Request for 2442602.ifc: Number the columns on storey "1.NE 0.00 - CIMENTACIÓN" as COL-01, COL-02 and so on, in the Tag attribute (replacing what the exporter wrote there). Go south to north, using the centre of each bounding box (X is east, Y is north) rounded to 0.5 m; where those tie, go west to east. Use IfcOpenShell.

First a look at what the model holds.

```python
import ifcopenshell
import ifcopenshell.util.element
import ifcopenshell.util.placement

model = ifcopenshell.open("2442602.ifc")
print(model.schema)
storey = next(s for s in model.by_type("IfcBuildingStorey") if s.Name == "1.NE 0.00 - CIMENTACIÓN")
columns = [e for e in ifcopenshell.util.element.get_decomposition(storey) if e.is_a("IfcColumn")]
for e in sorted(columns, key=lambda e: e.id()):
    origin = ifcopenshell.util.placement.get_local_placement(e.ObjectPlacement)[:3, 3]
    print(e.id(), e.Tag, e.Name, origin.round(2) + 0.0, sep=" | ")
```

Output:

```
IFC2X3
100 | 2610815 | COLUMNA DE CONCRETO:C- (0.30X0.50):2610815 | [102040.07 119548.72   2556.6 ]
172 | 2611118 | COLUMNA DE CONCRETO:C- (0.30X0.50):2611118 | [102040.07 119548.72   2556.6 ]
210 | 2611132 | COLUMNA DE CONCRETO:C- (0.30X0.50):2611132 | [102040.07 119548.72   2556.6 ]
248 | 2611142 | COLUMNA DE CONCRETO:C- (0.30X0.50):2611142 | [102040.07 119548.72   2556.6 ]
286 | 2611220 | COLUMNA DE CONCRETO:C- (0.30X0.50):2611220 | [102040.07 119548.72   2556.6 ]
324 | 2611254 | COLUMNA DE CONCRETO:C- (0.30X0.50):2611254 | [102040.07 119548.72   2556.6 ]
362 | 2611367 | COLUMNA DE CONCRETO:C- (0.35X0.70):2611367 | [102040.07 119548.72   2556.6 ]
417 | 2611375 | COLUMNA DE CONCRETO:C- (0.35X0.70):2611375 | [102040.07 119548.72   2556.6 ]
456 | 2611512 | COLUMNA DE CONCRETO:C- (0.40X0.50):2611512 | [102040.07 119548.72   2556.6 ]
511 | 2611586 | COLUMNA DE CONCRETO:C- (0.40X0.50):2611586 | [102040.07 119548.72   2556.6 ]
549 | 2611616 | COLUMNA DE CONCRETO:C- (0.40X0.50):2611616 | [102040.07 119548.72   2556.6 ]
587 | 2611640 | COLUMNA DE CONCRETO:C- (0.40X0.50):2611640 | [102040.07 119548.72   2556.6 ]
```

```python
import ifcopenshell
import ifcopenshell.geom
import ifcopenshell.util.element
import ifcopenshell.util.shape

model = ifcopenshell.open("2442602.ifc")
settings = ifcopenshell.geom.settings()
settings.set("use-world-coords", True)


def centre(element):
    shape = ifcopenshell.geom.create_shape(settings, element)
    return ifcopenshell.util.shape.get_bbox_centroid(shape.geometry)


storey = next(s for s in model.by_type("IfcBuildingStorey") if s.Name == "1.NE 0.00 - CIMENTACIÓN")
columns = [e for e in ifcopenshell.util.element.get_decomposition(storey) if e.is_a("IfcColumn")]

# Insertion points can sit at a corner or the storey origin, so sort by the geometry (in metres).
centres = {e: centre(e) for e in columns}
columns.sort(key=lambda e: (round(centres[e][1] / 0.5), centres[e][0]))

for i, e in enumerate(columns, start=1):
    number = f"COL-{i:02d}"
    e.Tag = number
    print(e.id(), number)

model.write("2442602_rev.ifc")
```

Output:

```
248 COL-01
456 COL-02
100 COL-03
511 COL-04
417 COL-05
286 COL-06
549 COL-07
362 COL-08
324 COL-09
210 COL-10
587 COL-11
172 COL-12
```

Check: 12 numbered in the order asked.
